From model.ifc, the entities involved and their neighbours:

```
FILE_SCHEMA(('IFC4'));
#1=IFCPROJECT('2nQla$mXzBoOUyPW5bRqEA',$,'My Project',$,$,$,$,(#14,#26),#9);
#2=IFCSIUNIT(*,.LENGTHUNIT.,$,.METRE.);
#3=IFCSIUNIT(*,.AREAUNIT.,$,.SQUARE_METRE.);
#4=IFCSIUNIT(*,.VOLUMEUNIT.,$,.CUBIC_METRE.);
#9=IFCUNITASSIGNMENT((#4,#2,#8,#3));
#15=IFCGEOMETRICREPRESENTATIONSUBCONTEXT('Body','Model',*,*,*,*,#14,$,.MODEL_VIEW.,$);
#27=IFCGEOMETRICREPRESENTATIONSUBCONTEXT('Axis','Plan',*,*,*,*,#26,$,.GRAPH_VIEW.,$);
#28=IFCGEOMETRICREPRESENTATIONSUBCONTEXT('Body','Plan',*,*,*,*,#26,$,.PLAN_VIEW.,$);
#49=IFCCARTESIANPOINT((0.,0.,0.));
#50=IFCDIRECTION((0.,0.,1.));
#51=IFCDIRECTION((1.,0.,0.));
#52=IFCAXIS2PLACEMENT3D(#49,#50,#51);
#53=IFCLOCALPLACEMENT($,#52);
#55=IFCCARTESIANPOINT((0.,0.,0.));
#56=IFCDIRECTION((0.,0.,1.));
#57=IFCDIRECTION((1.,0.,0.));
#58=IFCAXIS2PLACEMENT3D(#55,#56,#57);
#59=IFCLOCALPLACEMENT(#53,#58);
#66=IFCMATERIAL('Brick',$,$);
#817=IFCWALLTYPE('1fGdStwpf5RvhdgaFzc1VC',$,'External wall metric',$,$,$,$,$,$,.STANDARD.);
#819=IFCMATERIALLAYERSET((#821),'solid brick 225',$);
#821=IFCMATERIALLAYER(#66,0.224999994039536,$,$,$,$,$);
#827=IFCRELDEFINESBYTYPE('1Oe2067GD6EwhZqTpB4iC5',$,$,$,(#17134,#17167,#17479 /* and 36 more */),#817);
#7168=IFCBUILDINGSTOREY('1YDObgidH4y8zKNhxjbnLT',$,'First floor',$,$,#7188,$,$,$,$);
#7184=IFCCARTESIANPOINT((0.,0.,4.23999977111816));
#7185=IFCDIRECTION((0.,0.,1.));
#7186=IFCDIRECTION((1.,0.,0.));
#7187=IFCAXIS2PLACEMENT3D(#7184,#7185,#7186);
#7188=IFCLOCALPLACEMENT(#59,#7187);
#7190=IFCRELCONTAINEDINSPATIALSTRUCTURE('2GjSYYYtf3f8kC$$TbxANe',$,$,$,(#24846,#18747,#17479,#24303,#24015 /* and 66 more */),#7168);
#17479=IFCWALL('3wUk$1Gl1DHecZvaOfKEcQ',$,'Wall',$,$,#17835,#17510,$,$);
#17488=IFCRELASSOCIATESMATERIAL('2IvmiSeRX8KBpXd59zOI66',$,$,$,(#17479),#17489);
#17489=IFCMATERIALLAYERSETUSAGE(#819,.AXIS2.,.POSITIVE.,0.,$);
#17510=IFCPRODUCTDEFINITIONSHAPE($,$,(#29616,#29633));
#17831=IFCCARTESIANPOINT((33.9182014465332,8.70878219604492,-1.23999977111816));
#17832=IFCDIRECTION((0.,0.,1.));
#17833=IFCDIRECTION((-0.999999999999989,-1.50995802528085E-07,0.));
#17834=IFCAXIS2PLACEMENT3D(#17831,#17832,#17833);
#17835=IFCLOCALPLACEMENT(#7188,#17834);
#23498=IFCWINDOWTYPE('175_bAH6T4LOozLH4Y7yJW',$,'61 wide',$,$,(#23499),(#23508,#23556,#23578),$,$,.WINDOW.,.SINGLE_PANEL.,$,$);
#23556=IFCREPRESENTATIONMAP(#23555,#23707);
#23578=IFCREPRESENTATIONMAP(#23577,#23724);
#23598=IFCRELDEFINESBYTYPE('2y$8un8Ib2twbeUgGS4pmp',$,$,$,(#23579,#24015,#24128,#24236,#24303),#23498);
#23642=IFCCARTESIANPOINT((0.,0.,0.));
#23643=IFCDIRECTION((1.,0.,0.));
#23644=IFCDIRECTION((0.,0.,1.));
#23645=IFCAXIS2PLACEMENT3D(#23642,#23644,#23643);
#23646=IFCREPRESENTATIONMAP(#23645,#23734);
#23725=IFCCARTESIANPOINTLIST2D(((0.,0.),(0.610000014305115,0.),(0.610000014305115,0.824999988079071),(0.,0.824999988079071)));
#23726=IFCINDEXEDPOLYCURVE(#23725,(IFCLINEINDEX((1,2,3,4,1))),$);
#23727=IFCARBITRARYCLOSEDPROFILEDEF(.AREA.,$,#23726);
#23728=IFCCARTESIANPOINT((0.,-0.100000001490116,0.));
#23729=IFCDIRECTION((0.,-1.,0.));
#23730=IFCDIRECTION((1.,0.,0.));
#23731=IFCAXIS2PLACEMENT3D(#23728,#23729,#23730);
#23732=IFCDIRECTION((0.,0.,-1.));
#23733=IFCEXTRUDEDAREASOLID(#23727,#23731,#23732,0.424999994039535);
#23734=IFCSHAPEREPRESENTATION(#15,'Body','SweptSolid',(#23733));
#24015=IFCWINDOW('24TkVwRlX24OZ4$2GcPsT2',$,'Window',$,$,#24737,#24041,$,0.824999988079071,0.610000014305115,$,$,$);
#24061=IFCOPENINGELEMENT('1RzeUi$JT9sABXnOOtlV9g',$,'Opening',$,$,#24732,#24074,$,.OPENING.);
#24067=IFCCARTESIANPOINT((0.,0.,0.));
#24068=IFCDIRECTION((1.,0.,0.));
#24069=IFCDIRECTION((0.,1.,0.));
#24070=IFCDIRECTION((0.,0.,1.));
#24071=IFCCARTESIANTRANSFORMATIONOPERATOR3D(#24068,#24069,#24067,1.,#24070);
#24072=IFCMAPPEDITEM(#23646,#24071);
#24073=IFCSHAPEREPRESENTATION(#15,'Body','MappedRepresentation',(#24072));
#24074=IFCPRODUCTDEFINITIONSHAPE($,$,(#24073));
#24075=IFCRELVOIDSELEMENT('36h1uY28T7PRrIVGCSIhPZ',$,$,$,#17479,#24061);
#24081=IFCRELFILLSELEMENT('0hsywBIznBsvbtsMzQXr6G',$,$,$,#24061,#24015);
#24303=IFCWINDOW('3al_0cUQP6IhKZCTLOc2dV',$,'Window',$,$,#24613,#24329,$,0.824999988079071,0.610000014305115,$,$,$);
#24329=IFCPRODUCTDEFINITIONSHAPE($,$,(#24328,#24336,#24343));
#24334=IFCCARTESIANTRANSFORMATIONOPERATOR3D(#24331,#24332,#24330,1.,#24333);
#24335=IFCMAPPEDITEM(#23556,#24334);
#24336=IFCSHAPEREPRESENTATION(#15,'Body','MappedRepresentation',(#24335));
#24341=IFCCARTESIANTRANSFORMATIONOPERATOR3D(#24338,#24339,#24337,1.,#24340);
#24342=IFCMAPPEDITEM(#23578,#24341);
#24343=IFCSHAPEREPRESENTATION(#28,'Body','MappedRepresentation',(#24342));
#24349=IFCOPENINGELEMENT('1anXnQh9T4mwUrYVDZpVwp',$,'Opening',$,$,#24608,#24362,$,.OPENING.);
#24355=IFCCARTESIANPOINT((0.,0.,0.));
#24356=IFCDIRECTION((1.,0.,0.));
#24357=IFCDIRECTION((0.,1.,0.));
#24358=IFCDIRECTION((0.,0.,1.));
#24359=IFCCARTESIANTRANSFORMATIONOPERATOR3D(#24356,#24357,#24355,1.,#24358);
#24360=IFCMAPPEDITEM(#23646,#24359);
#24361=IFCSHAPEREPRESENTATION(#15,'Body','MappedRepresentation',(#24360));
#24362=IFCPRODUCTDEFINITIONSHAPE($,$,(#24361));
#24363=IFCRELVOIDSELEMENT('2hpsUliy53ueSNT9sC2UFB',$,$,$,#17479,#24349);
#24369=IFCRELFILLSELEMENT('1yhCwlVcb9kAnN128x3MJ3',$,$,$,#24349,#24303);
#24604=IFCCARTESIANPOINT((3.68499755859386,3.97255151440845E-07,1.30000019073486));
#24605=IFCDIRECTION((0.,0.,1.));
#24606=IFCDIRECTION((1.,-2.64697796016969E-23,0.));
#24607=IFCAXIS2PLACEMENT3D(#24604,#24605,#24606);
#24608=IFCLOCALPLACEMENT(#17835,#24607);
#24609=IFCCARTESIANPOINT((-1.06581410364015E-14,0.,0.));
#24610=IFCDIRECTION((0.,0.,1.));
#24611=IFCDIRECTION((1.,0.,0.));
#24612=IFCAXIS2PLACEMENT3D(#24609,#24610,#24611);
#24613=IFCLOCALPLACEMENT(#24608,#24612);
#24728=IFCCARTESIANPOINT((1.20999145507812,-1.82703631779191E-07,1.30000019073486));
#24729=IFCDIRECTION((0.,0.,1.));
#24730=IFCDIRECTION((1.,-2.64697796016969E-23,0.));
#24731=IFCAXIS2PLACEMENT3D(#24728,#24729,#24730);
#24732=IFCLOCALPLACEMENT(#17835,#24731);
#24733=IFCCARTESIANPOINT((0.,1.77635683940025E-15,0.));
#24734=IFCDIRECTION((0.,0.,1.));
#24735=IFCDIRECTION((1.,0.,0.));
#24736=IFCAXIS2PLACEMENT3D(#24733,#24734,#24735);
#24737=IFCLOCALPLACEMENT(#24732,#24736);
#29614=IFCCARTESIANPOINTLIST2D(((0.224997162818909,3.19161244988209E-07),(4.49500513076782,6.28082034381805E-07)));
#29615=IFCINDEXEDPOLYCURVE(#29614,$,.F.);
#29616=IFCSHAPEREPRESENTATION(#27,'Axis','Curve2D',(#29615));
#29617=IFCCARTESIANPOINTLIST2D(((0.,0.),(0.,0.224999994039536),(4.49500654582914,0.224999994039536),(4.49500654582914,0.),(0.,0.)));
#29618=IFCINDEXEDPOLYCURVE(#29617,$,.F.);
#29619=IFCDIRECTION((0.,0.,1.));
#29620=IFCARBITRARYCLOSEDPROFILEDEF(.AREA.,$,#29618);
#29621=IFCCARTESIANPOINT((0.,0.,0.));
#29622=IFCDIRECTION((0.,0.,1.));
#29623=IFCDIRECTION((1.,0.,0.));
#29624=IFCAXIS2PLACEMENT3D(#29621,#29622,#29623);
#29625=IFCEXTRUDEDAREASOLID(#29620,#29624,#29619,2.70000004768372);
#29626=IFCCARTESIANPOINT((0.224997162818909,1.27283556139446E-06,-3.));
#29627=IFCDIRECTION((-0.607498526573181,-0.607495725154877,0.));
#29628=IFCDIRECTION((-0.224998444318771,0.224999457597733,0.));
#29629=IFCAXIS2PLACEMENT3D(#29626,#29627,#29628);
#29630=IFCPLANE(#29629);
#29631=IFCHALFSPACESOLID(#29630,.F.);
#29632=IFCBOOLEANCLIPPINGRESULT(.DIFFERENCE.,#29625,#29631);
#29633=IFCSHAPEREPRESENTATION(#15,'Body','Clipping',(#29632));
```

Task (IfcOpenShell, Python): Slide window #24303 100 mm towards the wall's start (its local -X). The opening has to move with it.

```python
import ifcopenshell
import ifcopenshell.api.geometry
import ifcopenshell.util.placement

model = ifcopenshell.open("model.ifc")

window = model.by_id(24303)
opening = window.FillsVoids[0].RelatingOpeningElement
wall = opening.VoidsElements[0].RelatingBuildingElement

wall_matrix = ifcopenshell.util.placement.get_local_placement(wall.ObjectPlacement)
shift = wall_matrix[:3, 0] * -0.1
before = ifcopenshell.util.placement.get_local_placement(window.ObjectPlacement)[:3, 3].copy()

# The window is placed relative to its opening, so it follows when the opening moves.
matrix = ifcopenshell.util.placement.get_local_placement(opening.ObjectPlacement)
matrix[:3, 3] += shift
ifcopenshell.api.geometry.edit_object_placement(
    model, product=opening, matrix=matrix, is_si=False, should_transform_children=True
)

after = ifcopenshell.util.placement.get_local_placement(window.ObjectPlacement)[:3, 3]
print("window moved by", (after - before).round(3) + 0.0)

model.write("model-out.ifc")
```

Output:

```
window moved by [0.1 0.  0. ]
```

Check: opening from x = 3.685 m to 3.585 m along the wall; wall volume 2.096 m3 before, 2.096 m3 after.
